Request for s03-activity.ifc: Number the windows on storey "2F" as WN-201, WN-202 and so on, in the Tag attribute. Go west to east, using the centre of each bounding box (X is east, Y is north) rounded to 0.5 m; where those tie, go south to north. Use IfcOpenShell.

First a look at what the model holds.

```python
import ifcopenshell
import ifcopenshell.util.element
import ifcopenshell.util.placement

model = ifcopenshell.open("s03-activity.ifc")
print(model.schema)
storey = next(s for s in model.by_type("IfcBuildingStorey") if s.Name == "2F")
windows = [e for e in ifcopenshell.util.element.get_decomposition(storey) if e.is_a("IfcWindow")]
for e in sorted(windows, key=lambda e: e.id()):
    origin = ifcopenshell.util.placement.get_local_placement(e.ObjectPlacement)[:3, 3]
    print(e.id(), e.Tag, e.Name, origin.round(2) + 0.0, sep=" | ")
```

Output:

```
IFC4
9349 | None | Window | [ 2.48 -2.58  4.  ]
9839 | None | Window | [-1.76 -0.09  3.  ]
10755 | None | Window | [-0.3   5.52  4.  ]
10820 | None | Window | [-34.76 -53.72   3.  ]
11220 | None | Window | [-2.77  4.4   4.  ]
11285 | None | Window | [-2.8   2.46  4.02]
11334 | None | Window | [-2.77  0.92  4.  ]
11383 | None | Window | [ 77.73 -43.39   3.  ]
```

```python
import ifcopenshell
import ifcopenshell.geom
import ifcopenshell.util.element
import ifcopenshell.util.shape

model = ifcopenshell.open("s03-activity.ifc")
settings = ifcopenshell.geom.settings()
settings.set("use-world-coords", True)


def centre(element):
    shape = ifcopenshell.geom.create_shape(settings, element)
    return ifcopenshell.util.shape.get_bbox_centroid(shape.geometry)


storey = next(s for s in model.by_type("IfcBuildingStorey") if s.Name == "2F")
windows = [e for e in ifcopenshell.util.element.get_decomposition(storey) if e.is_a("IfcWindow")]

# Insertion points can sit at a corner or the storey origin, so sort by the geometry (in metres).
centres = {e: centre(e) for e in windows}
windows.sort(key=lambda e: (round(centres[e][0] / 0.5), centres[e][1]))

for i, e in enumerate(windows, start=1):
    number = f"WN-2{i:02d}"
    e.Tag = number
    print(e.id(), number)

model.write("s03-activity_updated.ifc")
```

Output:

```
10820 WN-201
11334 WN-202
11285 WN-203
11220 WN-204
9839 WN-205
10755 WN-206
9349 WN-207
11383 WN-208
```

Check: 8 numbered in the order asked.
